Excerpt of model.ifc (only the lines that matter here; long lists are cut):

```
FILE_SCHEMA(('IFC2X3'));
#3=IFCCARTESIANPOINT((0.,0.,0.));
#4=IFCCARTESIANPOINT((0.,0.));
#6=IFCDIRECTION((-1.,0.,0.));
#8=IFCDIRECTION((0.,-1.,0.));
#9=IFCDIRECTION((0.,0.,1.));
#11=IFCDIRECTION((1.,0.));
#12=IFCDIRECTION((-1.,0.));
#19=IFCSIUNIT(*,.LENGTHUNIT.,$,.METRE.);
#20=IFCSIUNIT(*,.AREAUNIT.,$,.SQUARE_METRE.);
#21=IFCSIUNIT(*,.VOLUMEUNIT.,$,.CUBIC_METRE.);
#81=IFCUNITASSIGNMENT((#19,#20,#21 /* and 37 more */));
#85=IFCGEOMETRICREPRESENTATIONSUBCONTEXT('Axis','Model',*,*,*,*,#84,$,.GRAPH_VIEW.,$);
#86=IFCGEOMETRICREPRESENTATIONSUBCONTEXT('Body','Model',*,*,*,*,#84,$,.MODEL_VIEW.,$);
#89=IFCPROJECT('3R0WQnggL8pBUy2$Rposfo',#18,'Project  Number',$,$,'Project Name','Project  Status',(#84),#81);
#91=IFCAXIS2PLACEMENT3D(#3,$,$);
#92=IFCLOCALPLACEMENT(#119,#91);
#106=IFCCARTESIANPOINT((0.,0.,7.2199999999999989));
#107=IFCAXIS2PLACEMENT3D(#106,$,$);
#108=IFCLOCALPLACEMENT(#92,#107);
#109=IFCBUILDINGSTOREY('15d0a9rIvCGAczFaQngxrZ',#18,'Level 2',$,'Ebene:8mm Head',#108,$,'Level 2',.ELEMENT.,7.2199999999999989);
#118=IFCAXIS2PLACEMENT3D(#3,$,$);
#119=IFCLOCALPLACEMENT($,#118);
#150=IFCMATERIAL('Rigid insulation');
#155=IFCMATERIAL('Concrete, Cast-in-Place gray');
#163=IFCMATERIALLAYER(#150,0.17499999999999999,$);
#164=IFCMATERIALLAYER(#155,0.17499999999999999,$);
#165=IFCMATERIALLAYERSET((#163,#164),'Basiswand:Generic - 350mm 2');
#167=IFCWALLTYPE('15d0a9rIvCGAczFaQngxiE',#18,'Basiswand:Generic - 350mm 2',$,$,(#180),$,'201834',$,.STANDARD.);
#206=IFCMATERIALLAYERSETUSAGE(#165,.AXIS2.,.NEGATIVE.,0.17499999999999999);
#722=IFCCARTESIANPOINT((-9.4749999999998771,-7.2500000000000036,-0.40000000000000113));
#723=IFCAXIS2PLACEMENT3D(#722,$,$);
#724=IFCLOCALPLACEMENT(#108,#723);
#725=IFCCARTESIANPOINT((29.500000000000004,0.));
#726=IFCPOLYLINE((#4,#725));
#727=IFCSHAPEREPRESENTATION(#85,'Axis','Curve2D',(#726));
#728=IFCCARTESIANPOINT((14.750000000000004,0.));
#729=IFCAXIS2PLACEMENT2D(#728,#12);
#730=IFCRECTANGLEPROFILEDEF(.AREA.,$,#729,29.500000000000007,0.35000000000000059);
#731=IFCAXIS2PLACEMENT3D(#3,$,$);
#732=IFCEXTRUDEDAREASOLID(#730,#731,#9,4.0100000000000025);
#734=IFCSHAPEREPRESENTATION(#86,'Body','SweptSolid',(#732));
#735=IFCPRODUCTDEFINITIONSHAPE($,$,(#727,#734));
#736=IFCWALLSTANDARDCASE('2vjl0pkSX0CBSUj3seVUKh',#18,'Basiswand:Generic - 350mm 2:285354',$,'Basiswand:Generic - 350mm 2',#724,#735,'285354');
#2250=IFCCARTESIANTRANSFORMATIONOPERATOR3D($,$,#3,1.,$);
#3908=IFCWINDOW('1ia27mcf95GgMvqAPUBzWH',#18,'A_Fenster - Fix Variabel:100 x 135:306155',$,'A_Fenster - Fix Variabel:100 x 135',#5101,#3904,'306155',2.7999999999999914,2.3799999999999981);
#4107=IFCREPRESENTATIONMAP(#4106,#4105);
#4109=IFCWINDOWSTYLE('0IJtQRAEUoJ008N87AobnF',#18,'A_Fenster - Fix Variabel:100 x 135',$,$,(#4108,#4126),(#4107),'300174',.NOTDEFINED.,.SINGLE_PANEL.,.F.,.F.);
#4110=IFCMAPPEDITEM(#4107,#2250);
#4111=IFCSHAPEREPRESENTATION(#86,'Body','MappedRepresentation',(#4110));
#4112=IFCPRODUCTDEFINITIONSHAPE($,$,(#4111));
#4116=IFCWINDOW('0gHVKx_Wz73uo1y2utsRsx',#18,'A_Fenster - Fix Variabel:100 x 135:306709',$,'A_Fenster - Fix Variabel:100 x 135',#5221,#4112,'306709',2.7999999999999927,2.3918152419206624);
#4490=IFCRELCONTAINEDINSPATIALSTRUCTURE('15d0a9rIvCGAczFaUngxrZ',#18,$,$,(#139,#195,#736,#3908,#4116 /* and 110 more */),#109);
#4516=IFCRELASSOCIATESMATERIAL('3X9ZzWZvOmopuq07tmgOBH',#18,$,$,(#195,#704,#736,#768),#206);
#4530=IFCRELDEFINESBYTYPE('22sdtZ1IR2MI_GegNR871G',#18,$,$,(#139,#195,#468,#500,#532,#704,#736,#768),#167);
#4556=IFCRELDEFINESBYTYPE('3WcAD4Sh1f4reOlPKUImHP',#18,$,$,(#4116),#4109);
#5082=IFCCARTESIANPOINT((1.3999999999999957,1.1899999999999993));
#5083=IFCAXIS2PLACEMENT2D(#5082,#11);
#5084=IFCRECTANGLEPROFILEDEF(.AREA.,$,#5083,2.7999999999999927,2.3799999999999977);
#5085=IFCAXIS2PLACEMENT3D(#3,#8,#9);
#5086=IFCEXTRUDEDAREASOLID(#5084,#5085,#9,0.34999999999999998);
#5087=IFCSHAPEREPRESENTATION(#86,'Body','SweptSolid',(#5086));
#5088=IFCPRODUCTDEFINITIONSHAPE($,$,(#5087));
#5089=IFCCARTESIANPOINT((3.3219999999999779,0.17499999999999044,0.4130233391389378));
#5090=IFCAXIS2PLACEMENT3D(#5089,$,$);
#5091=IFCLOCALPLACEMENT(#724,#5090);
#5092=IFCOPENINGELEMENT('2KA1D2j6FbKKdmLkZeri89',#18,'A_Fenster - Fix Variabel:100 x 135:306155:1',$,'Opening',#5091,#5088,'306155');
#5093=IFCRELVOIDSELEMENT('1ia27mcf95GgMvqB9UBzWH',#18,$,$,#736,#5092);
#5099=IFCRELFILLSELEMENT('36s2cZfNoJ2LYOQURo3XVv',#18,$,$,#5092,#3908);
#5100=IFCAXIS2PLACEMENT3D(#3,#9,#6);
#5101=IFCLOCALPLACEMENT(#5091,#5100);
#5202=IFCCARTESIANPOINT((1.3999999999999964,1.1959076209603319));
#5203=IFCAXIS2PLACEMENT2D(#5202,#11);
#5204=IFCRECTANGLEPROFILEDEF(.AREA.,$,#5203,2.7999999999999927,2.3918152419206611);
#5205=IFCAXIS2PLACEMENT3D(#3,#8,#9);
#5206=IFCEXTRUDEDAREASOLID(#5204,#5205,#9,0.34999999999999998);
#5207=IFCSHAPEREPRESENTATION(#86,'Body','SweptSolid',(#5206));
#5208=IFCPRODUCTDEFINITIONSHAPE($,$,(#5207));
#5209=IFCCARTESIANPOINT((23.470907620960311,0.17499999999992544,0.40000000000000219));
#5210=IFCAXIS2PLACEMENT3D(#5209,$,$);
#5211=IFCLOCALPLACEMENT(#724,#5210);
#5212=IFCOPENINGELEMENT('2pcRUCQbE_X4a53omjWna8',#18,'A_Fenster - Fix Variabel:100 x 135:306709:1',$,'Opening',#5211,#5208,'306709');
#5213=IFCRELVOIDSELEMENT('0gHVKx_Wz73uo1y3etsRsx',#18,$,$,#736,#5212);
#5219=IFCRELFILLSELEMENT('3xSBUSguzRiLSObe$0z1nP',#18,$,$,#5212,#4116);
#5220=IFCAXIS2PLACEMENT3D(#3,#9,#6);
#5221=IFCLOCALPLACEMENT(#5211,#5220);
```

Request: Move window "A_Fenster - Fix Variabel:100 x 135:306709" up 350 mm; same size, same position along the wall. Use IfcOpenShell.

```python
import numpy as np
import ifcopenshell
import ifcopenshell.api.geometry
import ifcopenshell.util.placement
import ifcopenshell.util.unit

model = ifcopenshell.open("model.ifc")
unit_scale = ifcopenshell.util.unit.calculate_unit_scale(model)

window = model.by_id(4116)
opening = window.FillsVoids[0].RelatingOpeningElement
dz = 0.35 / unit_scale

shift = np.array([0.0, 0.0, dz])
# The window is placed relative to its opening, so it follows when the opening moves.
matrix = ifcopenshell.util.placement.get_local_placement(opening.ObjectPlacement)
matrix[:3, 3] += shift
ifcopenshell.api.geometry.edit_object_placement(
    model, product=opening, matrix=matrix, is_si=False, should_transform_children=True
)

print(f"moved by {dz * unit_scale:+.3f} m")

model.write("model_edited.ifc")
```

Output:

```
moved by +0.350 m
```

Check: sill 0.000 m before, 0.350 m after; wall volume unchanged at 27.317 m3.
